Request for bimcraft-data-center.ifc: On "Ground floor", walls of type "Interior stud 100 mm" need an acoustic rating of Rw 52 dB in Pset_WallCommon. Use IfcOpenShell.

First a look at what the model holds.

```python
import ifcopenshell
import ifcopenshell.util.element

model = ifcopenshell.open("bimcraft-data-center.ifc")
print(model.schema)
storey = next(s for s in model.by_type("IfcBuildingStorey") if s.Name == "Ground floor")
walls = [e for e in ifcopenshell.util.element.get_decomposition(storey) if e.is_a("IfcWall")]
seen = {}
for e in walls:
    element_type = ifcopenshell.util.element.get_type(e)
    key = (element_type.Name if element_type != e and element_type else None, ifcopenshell.util.element.get_pset(e, "Pset_WallCommon", "AcousticRating"))
    seen[key] = seen.get(key, 0) + 1
for (name, value), count in sorted(seen.items(), key=str):
    print(count, "x", name, "|", value)
```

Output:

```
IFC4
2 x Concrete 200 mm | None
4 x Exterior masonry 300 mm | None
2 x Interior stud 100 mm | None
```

```python
import ifcopenshell
import ifcopenshell.api.pset
import ifcopenshell.util.element

model = ifcopenshell.open("bimcraft-data-center.ifc")

storey = next(s for s in model.by_type("IfcBuildingStorey") if s.Name == "Ground floor")
walls = [e for e in ifcopenshell.util.element.get_decomposition(storey) if e.is_a("IfcWall")]

count = 0
for e in walls:
    element_type = ifcopenshell.util.element.get_type(e)
    if element_type in (None, e) or element_type.Name != "Interior stud 100 mm":
        continue
    # add_pset returns the element's existing set when there is one.
    pset = ifcopenshell.api.pset.add_pset(model, product=e, name="Pset_WallCommon")
    ifcopenshell.api.pset.edit_pset(model, pset=pset, properties={"AcousticRating": "Rw 52 dB"})
    count += 1

print(count, "walls updated")

model.write("bimcraft-data-center_updated.ifc")
```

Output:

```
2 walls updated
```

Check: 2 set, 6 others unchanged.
